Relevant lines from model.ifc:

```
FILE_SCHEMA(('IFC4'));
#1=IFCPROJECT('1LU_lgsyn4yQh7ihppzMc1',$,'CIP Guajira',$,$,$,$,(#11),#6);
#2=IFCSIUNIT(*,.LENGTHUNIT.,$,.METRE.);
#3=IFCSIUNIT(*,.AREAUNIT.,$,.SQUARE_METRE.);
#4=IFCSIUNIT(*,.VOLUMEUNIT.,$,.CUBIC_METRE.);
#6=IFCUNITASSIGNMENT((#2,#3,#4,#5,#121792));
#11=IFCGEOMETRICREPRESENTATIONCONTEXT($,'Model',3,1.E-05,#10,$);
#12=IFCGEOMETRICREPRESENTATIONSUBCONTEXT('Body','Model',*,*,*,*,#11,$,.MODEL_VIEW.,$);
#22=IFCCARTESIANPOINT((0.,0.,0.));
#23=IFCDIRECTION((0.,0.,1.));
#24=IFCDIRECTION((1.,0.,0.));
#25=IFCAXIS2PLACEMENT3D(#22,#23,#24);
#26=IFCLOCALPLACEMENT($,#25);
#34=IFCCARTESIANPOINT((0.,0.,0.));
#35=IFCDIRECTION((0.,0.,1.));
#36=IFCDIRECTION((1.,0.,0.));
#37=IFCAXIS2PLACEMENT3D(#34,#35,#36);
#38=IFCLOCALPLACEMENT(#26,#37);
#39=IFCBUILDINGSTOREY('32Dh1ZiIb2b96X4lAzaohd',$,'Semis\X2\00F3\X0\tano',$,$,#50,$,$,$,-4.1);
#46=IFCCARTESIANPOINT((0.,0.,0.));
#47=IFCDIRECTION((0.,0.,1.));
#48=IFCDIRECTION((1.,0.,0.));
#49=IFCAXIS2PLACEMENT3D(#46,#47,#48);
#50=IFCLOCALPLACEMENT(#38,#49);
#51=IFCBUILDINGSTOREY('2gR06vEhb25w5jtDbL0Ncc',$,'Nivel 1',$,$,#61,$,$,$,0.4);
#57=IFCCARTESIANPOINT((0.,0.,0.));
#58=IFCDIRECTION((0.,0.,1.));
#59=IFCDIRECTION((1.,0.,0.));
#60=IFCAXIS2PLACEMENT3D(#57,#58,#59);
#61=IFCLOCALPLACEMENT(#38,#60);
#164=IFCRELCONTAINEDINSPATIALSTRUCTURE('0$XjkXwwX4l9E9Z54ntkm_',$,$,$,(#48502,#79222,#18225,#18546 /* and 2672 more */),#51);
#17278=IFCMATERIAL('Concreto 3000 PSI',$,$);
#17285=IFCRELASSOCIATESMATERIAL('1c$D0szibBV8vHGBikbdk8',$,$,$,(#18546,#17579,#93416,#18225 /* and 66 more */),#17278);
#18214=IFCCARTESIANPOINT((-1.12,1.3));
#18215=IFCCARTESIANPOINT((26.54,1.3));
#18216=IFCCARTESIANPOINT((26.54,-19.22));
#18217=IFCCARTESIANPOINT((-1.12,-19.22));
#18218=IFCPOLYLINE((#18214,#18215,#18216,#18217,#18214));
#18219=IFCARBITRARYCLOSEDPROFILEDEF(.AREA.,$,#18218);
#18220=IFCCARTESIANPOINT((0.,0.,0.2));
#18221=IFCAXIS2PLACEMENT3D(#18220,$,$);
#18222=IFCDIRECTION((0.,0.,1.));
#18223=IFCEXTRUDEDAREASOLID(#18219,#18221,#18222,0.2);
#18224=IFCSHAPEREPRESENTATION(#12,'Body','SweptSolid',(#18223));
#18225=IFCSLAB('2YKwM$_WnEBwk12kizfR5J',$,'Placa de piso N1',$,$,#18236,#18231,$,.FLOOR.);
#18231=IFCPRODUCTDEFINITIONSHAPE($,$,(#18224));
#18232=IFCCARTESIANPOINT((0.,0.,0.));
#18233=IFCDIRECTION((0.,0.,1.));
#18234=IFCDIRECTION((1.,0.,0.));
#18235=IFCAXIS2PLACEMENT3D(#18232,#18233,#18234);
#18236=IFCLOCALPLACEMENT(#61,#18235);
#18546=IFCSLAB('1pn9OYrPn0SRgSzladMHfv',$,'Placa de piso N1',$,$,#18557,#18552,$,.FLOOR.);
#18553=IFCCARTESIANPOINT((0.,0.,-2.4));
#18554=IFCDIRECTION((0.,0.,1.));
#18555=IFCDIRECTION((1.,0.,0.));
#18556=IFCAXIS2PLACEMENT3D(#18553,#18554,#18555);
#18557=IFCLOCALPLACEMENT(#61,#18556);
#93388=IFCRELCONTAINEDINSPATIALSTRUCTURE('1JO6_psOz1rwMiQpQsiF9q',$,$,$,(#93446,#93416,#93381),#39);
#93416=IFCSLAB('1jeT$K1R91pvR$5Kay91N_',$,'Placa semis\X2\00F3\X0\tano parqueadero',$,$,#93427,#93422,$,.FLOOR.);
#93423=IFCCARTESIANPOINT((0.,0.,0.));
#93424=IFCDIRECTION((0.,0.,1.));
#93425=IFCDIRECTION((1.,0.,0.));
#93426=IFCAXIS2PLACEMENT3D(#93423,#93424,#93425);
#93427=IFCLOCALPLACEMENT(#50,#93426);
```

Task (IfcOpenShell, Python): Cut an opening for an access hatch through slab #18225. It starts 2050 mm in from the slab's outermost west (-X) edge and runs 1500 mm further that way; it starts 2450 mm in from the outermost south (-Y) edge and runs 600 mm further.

```python
import numpy as np
import ifcopenshell
import ifcopenshell.api.feature
import ifcopenshell.api.geometry
import ifcopenshell.api.root
import ifcopenshell.geom
import ifcopenshell.util.placement
import ifcopenshell.util.representation
import ifcopenshell.util.shape
import ifcopenshell.util.unit

model = ifcopenshell.open("model.ifc")
unit_scale = ifcopenshell.util.unit.calculate_unit_scale(model)
settings = ifcopenshell.geom.settings()


def volume(element):
    """Net volume in cubic metres, openings subtracted."""
    shape = ifcopenshell.geom.create_shape(settings, element)
    return ifcopenshell.util.shape.get_volume(shape.geometry)


slab = model.by_guid("2YKwM$_WnEBwk12kizfR5J")
before = volume(slab)

# Extent in the slab's own axes, in metres. The edges named are its -X and -Y sides.
slab_shape = ifcopenshell.geom.create_shape(settings, slab)
vertices = ifcopenshell.util.shape.get_vertices(slab_shape.geometry)
x_min, y_min, bottom = vertices.min(axis=0)
top = vertices[:, 2].max()

opening = ifcopenshell.api.root.create_entity(model, ifc_class="IfcOpeningElement", name="Access hatch opening", predefined_type="OPENING")
context = ifcopenshell.util.representation.get_context(model, "Model", "Body", "MODEL_VIEW")
width, depth = 1.5, 0.6
outline = [(0.0, 0.0), (width, 0.0), (width, depth), (0.0, depth), (0.0, 0.0)]
# Overshoot both faces by 50 mm so the cut is clean.
shape = ifcopenshell.api.geometry.add_slab_representation(
    model, context=context, depth=top - bottom + 0.1, polyline=outline
)
ifcopenshell.api.geometry.assign_representation(model, product=opening, representation=shape)

matrix = ifcopenshell.util.placement.get_local_placement(slab.ObjectPlacement)
matrix[:, 3] = matrix @ np.append(np.array([x_min + 2.05, y_min + 2.45, bottom - 0.05]) / unit_scale, 1.0)
ifcopenshell.api.geometry.edit_object_placement(model, product=opening, matrix=matrix, is_si=False)
ifcopenshell.api.feature.add_feature(model, feature=opening, element=slab)

after = volume(slab)

print(f"slab volume {before:.3f} -> {after:.3f} m3")

model.write("model_rev.ifc")
```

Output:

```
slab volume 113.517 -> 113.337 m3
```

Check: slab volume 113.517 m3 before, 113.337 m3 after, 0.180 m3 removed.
